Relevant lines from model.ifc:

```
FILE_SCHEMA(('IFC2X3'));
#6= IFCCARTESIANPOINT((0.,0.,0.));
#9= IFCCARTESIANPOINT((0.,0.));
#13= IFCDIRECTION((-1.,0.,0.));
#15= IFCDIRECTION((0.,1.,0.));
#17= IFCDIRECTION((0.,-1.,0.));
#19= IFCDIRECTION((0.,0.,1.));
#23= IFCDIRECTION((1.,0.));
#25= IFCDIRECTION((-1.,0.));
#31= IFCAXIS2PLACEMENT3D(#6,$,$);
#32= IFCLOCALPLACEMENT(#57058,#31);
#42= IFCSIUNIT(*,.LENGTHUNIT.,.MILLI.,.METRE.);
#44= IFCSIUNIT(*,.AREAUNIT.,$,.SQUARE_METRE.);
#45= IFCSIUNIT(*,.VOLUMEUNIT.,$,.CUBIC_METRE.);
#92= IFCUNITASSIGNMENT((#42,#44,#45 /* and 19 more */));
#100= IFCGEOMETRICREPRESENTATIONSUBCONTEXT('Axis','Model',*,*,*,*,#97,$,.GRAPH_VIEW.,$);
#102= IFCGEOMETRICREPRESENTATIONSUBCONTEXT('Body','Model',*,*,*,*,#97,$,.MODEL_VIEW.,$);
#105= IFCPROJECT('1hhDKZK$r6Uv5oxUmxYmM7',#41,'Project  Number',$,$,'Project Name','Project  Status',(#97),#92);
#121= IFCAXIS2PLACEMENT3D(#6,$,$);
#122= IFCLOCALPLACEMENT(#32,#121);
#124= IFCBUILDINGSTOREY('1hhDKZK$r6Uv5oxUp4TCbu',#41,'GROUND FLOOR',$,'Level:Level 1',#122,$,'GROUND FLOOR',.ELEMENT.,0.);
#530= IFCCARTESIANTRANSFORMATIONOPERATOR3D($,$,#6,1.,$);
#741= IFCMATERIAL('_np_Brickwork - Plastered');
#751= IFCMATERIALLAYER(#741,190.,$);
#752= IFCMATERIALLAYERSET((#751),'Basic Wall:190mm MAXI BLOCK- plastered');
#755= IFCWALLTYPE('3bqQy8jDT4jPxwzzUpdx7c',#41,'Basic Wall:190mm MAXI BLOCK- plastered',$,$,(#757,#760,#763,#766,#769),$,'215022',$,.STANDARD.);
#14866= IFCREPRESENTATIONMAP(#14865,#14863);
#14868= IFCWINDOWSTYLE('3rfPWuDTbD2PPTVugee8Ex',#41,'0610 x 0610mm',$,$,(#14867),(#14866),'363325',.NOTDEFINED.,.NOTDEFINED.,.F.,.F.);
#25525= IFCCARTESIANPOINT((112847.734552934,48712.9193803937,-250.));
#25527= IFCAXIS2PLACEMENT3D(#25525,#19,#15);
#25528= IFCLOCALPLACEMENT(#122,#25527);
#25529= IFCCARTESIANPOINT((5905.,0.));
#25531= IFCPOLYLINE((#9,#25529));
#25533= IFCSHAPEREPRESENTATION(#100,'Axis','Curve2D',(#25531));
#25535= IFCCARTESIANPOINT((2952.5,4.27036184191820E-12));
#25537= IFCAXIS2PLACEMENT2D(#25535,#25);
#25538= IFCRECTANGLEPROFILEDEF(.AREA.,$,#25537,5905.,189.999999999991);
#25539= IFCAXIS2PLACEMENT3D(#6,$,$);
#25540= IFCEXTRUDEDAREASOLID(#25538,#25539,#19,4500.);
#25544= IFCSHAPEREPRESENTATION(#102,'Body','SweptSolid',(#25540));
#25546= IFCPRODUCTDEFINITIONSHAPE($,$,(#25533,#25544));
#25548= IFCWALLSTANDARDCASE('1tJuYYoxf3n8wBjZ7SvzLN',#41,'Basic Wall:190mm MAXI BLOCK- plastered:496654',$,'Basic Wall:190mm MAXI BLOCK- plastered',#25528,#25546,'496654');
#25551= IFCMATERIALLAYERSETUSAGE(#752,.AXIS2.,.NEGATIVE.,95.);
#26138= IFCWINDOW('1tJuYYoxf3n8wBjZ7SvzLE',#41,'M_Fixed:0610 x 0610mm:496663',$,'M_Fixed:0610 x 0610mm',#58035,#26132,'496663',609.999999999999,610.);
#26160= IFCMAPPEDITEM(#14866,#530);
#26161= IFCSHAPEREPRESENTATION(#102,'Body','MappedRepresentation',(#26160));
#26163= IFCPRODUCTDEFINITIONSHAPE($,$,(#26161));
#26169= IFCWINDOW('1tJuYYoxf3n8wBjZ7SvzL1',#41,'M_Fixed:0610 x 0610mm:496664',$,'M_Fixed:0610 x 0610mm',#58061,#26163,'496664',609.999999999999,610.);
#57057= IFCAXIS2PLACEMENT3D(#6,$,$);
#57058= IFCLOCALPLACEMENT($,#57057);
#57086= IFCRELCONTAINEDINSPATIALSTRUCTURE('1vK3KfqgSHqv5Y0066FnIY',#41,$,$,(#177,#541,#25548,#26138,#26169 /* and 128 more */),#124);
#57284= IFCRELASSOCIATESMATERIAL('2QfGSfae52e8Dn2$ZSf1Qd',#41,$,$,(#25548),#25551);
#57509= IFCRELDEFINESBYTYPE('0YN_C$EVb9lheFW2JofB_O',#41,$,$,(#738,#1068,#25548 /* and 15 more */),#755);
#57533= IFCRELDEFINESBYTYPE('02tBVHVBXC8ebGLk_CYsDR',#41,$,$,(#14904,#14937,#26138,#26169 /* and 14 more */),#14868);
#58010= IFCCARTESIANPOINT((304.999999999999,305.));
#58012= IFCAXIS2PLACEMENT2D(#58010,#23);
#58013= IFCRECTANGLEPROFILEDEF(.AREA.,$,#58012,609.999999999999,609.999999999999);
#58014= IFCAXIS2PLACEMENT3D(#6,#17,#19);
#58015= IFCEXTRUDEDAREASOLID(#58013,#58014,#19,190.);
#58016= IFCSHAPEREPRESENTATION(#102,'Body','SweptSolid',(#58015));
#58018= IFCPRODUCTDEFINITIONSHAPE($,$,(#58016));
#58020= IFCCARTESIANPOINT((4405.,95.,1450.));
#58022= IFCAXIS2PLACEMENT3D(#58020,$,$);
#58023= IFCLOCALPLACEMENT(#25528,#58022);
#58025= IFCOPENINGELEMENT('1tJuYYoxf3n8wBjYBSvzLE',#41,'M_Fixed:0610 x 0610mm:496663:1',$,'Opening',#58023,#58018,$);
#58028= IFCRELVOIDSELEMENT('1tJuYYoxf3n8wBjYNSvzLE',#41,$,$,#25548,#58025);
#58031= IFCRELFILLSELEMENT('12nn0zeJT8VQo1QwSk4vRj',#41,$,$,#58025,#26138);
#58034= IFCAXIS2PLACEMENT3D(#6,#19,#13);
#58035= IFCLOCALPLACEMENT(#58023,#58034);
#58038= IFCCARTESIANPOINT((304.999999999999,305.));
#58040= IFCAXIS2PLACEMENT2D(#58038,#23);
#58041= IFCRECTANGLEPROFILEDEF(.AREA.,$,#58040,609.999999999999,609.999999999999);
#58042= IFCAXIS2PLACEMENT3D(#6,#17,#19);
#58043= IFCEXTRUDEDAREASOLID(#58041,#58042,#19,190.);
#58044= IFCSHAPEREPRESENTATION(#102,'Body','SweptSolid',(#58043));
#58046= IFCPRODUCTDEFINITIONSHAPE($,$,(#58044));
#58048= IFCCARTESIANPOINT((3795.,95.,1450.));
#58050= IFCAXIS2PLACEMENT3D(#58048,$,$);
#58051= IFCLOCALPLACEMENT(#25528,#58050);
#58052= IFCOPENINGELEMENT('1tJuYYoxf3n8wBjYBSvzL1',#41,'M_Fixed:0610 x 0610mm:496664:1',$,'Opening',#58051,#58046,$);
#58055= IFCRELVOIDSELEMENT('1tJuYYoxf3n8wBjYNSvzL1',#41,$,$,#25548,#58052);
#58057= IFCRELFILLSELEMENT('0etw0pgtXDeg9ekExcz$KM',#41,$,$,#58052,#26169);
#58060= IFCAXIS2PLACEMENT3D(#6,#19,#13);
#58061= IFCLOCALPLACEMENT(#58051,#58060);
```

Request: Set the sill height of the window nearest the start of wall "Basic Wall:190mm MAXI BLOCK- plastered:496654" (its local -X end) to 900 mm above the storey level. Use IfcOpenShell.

```python
import numpy as np
import ifcopenshell
import ifcopenshell.api.geometry
import ifcopenshell.geom
import ifcopenshell.util.element
import ifcopenshell.util.placement
import ifcopenshell.util.shape
import ifcopenshell.util.unit

model = ifcopenshell.open("model.ifc")
unit_scale = ifcopenshell.util.unit.calculate_unit_scale(model)

window = model.by_id(26169)
opening = window.FillsVoids[0].RelatingOpeningElement
storey = ifcopenshell.util.element.get_container(window, ifc_class="IfcBuildingStorey")
level = ifcopenshell.util.placement.get_local_placement(storey.ObjectPlacement)[2, 3]

# The opening's origin need not be at the sill, so measure its lowest point.
shape = ifcopenshell.geom.create_shape(ifcopenshell.geom.settings(), opening)
bottom = ifcopenshell.util.shape.get_shape_bottom_elevation(shape, shape.geometry) / unit_scale
dz = level + 900.0 - bottom

shift = np.array([0.0, 0.0, dz])
# The window is placed relative to its opening, so it follows when the opening moves.
matrix = ifcopenshell.util.placement.get_local_placement(opening.ObjectPlacement)
matrix[:3, 3] += shift
ifcopenshell.api.geometry.edit_object_placement(
    model, product=opening, matrix=matrix, is_si=False, should_transform_children=True
)

print(f"moved by {dz * unit_scale:+.3f} m")

model.write("model-out.ifc")
```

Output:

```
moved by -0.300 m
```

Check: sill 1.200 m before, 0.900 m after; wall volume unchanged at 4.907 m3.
